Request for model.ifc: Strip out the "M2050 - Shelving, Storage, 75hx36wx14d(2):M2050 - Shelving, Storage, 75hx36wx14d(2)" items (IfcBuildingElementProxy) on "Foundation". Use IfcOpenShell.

First a look at what the model holds.

```python
import ifcopenshell
import ifcopenshell.util.element

model = ifcopenshell.open("model.ifc")
print(model.schema)
storey = next(s for s in model.by_type("IfcBuildingStorey") if s.Name == "Foundation")
proxies = [e for e in ifcopenshell.util.element.get_decomposition(storey) if e.is_a("IfcBuildingElementProxy")]
seen = {}
for e in proxies:
    element_type = ifcopenshell.util.element.get_type(e)
    name = element_type.Name if element_type not in (None, e) else None
    seen[name] = seen.get(name, 0) + 1
for name, count in sorted(seen.items(), key=str):
    print(count, "x", name)
```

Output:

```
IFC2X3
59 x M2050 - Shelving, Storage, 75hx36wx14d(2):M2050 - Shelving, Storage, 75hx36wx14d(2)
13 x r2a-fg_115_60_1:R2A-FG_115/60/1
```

```python
import ifcopenshell
import ifcopenshell.api.root
import ifcopenshell.util.element

model = ifcopenshell.open("model.ifc")

storey = next(s for s in model.by_type("IfcBuildingStorey") if s.Name == "Foundation")
proxies = [e for e in ifcopenshell.util.element.get_decomposition(storey) if e.is_a("IfcBuildingElementProxy")]
targets = [e for e in proxies if (t := ifcopenshell.util.element.get_type(e)) not in (None, e) and t.Name == "M2050 - Shelving, Storage, 75hx36wx14d(2):M2050 - Shelving, Storage, 75hx36wx14d(2)"]

for e in targets:
    ifcopenshell.api.root.remove_product(model, product=e)
print(len(targets), "removed")

model.write("model_v2.ifc")
```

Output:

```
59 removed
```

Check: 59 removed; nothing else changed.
